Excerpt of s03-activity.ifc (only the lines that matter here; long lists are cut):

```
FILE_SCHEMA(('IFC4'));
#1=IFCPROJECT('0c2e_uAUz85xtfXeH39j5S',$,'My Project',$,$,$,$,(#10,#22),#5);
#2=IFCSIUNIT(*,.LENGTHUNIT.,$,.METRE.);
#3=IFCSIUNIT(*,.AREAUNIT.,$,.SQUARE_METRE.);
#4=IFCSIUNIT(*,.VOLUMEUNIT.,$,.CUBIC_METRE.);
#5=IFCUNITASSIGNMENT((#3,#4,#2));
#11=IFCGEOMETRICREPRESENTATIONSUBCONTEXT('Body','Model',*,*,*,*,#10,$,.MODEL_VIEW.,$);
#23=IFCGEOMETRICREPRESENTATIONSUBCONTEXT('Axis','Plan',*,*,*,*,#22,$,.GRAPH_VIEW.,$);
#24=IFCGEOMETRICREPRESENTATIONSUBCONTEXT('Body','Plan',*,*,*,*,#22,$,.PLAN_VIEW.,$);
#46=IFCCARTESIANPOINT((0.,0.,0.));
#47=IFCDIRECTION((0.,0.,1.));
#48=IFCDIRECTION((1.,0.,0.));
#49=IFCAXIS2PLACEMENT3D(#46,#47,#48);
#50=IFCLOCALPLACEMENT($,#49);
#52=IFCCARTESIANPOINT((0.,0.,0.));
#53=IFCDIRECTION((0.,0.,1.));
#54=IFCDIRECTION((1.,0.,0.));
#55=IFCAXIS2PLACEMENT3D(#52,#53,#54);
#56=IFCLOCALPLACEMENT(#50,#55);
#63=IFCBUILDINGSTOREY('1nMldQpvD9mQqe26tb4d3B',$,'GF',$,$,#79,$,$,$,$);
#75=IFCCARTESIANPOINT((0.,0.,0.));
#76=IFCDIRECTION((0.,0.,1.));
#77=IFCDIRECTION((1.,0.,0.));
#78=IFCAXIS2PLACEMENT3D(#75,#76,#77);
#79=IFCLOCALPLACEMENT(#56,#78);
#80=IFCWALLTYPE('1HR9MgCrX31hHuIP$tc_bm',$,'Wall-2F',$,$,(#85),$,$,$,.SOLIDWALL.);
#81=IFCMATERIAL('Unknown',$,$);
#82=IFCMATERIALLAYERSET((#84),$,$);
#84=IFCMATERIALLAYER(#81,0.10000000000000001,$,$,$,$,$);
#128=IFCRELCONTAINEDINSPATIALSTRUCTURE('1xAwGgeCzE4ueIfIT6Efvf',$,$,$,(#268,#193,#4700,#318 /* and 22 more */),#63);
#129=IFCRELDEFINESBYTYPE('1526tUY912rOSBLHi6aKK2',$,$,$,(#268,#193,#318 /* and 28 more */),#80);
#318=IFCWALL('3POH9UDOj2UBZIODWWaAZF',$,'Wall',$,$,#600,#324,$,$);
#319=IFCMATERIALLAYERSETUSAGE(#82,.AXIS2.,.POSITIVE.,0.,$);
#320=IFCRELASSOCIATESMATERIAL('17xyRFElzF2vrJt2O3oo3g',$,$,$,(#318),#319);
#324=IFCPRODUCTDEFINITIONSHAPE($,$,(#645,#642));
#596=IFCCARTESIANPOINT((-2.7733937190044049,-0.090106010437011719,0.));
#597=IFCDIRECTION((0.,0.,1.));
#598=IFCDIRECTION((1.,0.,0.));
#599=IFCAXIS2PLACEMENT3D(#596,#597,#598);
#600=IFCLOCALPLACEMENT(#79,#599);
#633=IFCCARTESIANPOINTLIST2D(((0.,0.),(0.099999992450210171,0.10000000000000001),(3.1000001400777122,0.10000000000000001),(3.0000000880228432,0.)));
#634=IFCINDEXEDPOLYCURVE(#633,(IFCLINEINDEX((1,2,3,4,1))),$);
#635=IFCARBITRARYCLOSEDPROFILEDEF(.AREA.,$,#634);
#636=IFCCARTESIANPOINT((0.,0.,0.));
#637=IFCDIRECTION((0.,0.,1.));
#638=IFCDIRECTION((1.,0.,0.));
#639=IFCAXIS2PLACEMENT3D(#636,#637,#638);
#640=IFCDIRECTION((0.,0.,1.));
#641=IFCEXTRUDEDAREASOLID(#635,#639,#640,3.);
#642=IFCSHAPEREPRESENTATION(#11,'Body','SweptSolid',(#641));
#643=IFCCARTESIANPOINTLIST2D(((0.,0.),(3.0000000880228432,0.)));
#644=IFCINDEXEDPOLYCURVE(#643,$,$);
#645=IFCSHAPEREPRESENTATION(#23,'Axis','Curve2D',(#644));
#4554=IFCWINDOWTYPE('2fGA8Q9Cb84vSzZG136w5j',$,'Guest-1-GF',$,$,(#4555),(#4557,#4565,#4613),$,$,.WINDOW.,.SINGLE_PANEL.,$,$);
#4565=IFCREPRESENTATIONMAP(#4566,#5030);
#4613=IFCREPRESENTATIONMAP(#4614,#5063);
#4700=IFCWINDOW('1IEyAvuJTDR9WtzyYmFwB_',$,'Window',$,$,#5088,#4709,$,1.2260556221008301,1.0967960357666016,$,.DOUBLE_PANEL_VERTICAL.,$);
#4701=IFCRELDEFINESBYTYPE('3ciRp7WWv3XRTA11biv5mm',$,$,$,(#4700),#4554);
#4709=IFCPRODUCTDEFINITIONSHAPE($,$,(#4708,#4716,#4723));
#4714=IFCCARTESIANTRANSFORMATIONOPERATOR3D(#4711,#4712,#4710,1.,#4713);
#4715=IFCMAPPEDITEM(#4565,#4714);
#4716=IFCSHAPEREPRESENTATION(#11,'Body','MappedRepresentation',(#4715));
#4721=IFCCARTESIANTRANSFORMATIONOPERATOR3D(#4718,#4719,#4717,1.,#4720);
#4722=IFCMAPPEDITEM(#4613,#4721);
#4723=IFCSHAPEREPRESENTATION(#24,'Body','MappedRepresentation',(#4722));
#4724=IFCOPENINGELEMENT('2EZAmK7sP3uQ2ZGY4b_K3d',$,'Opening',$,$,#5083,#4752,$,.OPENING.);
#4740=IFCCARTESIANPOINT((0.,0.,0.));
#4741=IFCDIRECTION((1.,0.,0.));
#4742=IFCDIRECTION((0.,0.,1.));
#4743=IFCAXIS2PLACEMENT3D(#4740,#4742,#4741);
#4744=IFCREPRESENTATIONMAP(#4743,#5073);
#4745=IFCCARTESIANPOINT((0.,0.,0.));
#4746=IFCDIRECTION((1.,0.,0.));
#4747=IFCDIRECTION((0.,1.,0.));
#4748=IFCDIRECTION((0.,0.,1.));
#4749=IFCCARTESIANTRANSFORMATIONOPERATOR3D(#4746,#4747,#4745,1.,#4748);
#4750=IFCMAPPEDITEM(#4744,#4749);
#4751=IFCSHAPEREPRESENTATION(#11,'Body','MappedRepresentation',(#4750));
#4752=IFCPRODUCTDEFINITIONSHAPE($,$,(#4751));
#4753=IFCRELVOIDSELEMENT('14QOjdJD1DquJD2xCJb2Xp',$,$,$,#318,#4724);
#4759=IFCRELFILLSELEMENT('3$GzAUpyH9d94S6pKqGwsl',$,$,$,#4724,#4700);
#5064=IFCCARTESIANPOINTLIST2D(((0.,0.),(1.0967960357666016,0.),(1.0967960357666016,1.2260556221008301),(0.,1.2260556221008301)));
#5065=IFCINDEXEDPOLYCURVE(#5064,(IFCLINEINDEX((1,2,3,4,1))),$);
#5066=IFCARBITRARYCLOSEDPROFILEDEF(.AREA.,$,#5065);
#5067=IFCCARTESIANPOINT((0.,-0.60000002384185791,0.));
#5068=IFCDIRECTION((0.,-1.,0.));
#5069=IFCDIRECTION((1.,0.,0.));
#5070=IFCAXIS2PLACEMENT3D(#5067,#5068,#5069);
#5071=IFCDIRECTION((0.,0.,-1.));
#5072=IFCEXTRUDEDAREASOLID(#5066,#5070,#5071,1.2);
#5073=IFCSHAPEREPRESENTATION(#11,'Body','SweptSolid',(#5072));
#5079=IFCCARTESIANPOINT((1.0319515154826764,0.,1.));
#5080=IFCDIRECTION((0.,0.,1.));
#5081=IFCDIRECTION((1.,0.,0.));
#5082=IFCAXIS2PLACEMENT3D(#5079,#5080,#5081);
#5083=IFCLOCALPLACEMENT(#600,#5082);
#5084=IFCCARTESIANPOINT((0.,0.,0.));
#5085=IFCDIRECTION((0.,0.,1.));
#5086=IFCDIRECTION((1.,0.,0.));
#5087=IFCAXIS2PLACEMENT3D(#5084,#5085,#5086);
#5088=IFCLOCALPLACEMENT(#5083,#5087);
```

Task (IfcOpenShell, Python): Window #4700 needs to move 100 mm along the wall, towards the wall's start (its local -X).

```python
import ifcopenshell
import ifcopenshell.api.geometry
import ifcopenshell.util.placement
import ifcopenshell.util.unit

model = ifcopenshell.open("s03-activity.ifc")
unit_scale = ifcopenshell.util.unit.calculate_unit_scale(model)

window = model.by_guid("1IEyAvuJTDR9WtzyYmFwB_")
opening = window.FillsVoids[0].RelatingOpeningElement
wall = opening.VoidsElements[0].RelatingBuildingElement

wall_matrix = ifcopenshell.util.placement.get_local_placement(wall.ObjectPlacement)
shift = wall_matrix[:3, 0] * -0.1 / unit_scale
before = ifcopenshell.util.placement.get_local_placement(window.ObjectPlacement)[:3, 3].copy()

# The window is placed relative to its opening, so it follows when the opening moves.
matrix = ifcopenshell.util.placement.get_local_placement(opening.ObjectPlacement)
matrix[:3, 3] += shift
ifcopenshell.api.geometry.edit_object_placement(
    model, product=opening, matrix=matrix, is_si=False, should_transform_children=True
)

after = ifcopenshell.util.placement.get_local_placement(window.ObjectPlacement)[:3, 3]
print("window moved by", (after - before).round(3) + 0.0)

model.write("s03-activity_edited.ifc")
```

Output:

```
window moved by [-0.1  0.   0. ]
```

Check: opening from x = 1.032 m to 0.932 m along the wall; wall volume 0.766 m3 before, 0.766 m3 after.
